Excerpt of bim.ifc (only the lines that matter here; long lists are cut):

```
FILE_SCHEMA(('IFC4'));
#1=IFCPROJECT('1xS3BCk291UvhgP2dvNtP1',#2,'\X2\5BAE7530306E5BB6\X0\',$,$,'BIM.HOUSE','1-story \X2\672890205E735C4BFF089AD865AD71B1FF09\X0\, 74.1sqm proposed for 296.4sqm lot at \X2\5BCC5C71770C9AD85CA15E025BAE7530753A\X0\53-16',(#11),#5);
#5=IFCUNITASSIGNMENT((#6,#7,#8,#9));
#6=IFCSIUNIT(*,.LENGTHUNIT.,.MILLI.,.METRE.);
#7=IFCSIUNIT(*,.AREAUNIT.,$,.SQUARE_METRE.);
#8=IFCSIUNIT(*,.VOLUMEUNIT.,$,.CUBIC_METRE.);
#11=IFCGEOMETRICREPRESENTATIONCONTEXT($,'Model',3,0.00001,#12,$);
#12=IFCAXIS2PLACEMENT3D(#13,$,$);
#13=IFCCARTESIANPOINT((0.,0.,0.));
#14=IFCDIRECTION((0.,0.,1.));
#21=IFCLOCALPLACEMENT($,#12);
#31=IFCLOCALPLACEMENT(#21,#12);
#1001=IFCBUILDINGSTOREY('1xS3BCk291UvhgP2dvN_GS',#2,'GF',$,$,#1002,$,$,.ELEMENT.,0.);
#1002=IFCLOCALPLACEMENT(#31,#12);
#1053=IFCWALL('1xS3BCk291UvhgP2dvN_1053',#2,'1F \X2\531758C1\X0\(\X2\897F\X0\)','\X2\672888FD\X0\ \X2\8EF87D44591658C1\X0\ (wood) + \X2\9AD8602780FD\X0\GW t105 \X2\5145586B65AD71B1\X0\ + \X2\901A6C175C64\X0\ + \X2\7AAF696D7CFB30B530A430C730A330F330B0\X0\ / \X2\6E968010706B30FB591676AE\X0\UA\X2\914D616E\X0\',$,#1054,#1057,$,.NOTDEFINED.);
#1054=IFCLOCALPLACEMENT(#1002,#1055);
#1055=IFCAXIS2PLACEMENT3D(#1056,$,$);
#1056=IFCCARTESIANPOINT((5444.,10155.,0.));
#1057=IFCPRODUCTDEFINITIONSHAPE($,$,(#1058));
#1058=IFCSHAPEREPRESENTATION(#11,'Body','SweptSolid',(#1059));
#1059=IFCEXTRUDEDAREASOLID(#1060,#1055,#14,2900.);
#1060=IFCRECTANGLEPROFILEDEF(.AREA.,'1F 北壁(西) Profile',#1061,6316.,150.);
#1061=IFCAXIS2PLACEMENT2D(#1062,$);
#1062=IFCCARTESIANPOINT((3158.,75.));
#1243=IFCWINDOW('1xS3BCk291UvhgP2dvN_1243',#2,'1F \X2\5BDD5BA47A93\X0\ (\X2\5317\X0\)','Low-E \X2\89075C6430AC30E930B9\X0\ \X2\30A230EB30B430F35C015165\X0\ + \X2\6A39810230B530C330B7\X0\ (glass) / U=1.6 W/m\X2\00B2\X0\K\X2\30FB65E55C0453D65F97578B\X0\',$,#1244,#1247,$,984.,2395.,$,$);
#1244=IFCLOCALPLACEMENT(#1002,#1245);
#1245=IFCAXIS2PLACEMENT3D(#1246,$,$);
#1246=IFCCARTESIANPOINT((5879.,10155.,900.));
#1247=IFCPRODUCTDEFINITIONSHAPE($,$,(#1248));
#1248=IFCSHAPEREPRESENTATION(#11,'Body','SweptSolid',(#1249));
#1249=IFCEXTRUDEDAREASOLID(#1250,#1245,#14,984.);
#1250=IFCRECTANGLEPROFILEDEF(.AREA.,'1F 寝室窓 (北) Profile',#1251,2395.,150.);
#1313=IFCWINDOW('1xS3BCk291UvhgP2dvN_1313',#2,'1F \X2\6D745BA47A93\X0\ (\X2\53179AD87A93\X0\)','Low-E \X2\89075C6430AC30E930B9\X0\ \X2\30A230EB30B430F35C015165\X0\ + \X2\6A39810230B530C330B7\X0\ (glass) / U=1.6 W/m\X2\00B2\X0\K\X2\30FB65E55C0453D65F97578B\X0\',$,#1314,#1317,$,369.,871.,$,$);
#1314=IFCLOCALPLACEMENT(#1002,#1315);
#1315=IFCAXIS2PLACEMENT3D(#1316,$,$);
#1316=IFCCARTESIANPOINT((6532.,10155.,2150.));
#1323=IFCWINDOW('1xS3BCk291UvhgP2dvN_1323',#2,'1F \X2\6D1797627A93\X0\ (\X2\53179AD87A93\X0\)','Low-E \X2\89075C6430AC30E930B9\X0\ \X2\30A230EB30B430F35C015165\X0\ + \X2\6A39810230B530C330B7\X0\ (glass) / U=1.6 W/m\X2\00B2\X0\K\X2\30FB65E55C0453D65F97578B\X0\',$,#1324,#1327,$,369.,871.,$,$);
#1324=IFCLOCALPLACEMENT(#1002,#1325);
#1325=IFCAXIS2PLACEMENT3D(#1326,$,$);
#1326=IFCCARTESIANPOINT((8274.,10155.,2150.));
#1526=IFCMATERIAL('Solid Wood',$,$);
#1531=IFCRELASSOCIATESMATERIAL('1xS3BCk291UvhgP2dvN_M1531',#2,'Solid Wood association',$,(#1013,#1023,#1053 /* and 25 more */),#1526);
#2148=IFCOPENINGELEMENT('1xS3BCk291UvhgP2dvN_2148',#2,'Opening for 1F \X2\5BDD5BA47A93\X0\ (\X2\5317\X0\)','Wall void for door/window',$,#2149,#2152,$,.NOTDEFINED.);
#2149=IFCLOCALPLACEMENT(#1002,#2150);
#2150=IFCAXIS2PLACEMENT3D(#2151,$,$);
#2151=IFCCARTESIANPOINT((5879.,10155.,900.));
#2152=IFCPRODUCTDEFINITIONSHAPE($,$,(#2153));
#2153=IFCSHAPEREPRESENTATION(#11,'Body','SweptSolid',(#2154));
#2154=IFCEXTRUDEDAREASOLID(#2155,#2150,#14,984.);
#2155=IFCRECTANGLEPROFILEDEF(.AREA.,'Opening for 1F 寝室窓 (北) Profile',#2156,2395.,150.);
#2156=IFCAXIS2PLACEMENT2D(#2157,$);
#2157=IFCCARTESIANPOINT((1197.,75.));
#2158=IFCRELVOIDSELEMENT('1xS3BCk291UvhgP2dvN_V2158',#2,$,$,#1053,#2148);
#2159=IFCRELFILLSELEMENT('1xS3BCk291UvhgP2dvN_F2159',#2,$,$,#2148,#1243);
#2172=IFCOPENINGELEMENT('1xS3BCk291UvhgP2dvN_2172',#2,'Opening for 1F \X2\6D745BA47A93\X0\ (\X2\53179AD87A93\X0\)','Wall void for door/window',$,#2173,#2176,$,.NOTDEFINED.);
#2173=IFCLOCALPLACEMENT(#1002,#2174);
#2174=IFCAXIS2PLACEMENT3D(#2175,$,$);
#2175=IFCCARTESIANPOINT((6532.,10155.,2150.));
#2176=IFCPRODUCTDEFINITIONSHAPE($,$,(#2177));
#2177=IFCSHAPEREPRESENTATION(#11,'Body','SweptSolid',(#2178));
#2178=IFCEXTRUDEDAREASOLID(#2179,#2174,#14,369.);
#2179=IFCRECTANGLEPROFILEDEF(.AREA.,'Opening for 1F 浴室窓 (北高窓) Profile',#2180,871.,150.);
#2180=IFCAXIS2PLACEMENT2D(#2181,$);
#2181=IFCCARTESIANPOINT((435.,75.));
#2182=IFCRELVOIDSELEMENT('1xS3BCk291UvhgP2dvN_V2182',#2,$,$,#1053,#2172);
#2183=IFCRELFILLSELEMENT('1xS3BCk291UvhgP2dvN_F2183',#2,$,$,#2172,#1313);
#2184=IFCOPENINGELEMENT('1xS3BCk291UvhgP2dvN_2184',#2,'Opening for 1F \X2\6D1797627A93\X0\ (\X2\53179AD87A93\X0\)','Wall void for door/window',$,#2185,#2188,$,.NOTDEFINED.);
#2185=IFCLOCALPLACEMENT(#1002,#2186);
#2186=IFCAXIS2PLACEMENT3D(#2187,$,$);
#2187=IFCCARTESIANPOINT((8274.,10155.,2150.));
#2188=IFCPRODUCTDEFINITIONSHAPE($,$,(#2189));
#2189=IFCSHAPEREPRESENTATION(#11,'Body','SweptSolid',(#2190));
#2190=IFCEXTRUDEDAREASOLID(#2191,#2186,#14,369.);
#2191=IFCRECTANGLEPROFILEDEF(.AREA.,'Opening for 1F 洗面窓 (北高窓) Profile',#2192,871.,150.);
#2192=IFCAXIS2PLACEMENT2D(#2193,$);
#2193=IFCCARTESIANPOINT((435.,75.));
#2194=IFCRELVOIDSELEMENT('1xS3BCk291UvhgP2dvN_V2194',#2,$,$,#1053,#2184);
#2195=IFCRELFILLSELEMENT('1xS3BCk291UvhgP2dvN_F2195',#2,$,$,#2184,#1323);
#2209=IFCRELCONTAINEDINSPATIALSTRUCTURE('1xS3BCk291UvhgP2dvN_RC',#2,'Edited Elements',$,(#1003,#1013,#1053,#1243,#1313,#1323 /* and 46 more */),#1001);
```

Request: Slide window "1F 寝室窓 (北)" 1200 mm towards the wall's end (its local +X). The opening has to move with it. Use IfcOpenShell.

```python
import ifcopenshell
import ifcopenshell.api.geometry
import ifcopenshell.util.placement

model = ifcopenshell.open("bim.ifc")

window = model.by_guid("1xS3BCk291UvhgP2dvN_1243")
opening = window.FillsVoids[0].RelatingOpeningElement
wall = opening.VoidsElements[0].RelatingBuildingElement

wall_matrix = ifcopenshell.util.placement.get_local_placement(wall.ObjectPlacement)
shift = wall_matrix[:3, 0] * 1200.0
before = ifcopenshell.util.placement.get_local_placement(window.ObjectPlacement)[:3, 3].copy()

# The window is not placed relative to its opening, so move both.
for product in (opening, window):
    matrix = ifcopenshell.util.placement.get_local_placement(product.ObjectPlacement)
    matrix[:3, 3] += shift
    ifcopenshell.api.geometry.edit_object_placement(model, product=product, matrix=matrix, is_si=False)

after = ifcopenshell.util.placement.get_local_placement(window.ObjectPlacement)[:3, 3]
print("window moved by", (after - before).round(3) + 0.0)

model.write("bim_rev.ifc")
```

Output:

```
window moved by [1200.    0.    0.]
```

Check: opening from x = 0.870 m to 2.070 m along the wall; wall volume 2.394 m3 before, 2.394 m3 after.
